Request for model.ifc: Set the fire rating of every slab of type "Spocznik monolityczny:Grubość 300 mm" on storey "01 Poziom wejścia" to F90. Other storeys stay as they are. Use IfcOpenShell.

First a look at what the model holds.

```python
import ifcopenshell
import ifcopenshell.util.element

model = ifcopenshell.open("model.ifc")
print(model.schema)
storey = next(s for s in model.by_type("IfcBuildingStorey") if s.Name == "01 Poziom wejścia")
slabs = [e for e in ifcopenshell.util.element.get_decomposition(storey) if e.is_a("IfcSlab")]
seen = {}
for e in slabs:
    element_type = ifcopenshell.util.element.get_type(e)
    key = (element_type.Name if element_type != e and element_type else None, ifcopenshell.util.element.get_pset(e, "Pset_SlabCommon", "FireRating"))
    seen[key] = seen.get(key, 0) + 1
for (name, value), count in sorted(seen.items(), key=str):
    print(count, "x", name, "|", value)
```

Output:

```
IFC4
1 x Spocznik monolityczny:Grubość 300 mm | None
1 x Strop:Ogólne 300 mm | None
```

```python
import ifcopenshell
import ifcopenshell.api.pset
import ifcopenshell.util.element

model = ifcopenshell.open("model.ifc")

storey = next(s for s in model.by_type("IfcBuildingStorey") if s.Name == "01 Poziom wejścia")
slabs = [e for e in ifcopenshell.util.element.get_decomposition(storey) if e.is_a("IfcSlab")]

count = 0
for e in slabs:
    element_type = ifcopenshell.util.element.get_type(e)
    if element_type in (None, e) or element_type.Name != "Spocznik monolityczny:Grubość 300 mm":
        continue
    # add_pset returns the element's existing set when there is one.
    pset = ifcopenshell.api.pset.add_pset(model, product=e, name="Pset_SlabCommon")
    ifcopenshell.api.pset.edit_pset(model, pset=pset, properties={"FireRating": "F90"})
    count += 1

print(count, "slabs updated")

model.write("model-out.ifc")
```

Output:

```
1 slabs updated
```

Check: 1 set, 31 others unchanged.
